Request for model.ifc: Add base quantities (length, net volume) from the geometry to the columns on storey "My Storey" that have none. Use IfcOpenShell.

First a look at what the model holds.

```python
import ifcopenshell
import ifcopenshell.util.element
import ifcopenshell.util.unit

model = ifcopenshell.open("model.ifc")
print(model.schema)
for unit_type in ("LENGTHUNIT", "AREAUNIT", "VOLUMEUNIT"):
    print(unit_type, ifcopenshell.util.unit.calculate_unit_scale(model, unit_type))
storey = next(s for s in model.by_type("IfcBuildingStorey") if s.Name == "My Storey")
columns = [e for e in ifcopenshell.util.element.get_decomposition(storey) if e.is_a("IfcColumn")]
for e in sorted(columns, key=lambda e: e.id()):
    print(e.id(), e.is_a(), e.Name, list(ifcopenshell.util.element.get_psets(e, qtos_only=True)), sep=" | ")
```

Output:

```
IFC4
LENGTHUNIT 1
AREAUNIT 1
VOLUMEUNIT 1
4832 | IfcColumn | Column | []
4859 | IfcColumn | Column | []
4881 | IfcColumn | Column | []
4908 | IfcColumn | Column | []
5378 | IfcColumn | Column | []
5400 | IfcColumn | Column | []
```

```python
import ifcopenshell
import ifcopenshell.api.pset
import ifcopenshell.geom
import ifcopenshell.util.element
import ifcopenshell.util.shape
import ifcopenshell.util.unit

model = ifcopenshell.open("model.ifc")
unit_scale = ifcopenshell.util.unit.calculate_unit_scale(model)
volume_scale = ifcopenshell.util.unit.calculate_unit_scale(model, "VOLUMEUNIT")
settings = ifcopenshell.geom.settings()

storey = next(s for s in model.by_type("IfcBuildingStorey") if s.Name == "My Storey")
columns = [e for e in ifcopenshell.util.element.get_decomposition(storey) if e.is_a("IfcColumn")]

for e in sorted(columns, key=lambda e: e.id()):
    if ifcopenshell.util.element.get_psets(e, qtos_only=True, should_inherit=False):
        continue
    # Geometry comes back in metres, in the element's own axes.
    shape = ifcopenshell.geom.create_shape(settings, e)
    values = {
        "Length": ifcopenshell.util.shape.get_z(shape.geometry) / unit_scale,
        "NetVolume": ifcopenshell.util.shape.get_volume(shape.geometry) / volume_scale,
    }
    qto = ifcopenshell.api.pset.add_qto(model, product=e, name="Qto_ColumnBaseQuantities")
    ifcopenshell.api.pset.edit_qto(model, qto=qto, properties=values)
    print(e.id(), {k: round(v, 3) for k, v in values.items()})

model.write("model_rev.ifc")
```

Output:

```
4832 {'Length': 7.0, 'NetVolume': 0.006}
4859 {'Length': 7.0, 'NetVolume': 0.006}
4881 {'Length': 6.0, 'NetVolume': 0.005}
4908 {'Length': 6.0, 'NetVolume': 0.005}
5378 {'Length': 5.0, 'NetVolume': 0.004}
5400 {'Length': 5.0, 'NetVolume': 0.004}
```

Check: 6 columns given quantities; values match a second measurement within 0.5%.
